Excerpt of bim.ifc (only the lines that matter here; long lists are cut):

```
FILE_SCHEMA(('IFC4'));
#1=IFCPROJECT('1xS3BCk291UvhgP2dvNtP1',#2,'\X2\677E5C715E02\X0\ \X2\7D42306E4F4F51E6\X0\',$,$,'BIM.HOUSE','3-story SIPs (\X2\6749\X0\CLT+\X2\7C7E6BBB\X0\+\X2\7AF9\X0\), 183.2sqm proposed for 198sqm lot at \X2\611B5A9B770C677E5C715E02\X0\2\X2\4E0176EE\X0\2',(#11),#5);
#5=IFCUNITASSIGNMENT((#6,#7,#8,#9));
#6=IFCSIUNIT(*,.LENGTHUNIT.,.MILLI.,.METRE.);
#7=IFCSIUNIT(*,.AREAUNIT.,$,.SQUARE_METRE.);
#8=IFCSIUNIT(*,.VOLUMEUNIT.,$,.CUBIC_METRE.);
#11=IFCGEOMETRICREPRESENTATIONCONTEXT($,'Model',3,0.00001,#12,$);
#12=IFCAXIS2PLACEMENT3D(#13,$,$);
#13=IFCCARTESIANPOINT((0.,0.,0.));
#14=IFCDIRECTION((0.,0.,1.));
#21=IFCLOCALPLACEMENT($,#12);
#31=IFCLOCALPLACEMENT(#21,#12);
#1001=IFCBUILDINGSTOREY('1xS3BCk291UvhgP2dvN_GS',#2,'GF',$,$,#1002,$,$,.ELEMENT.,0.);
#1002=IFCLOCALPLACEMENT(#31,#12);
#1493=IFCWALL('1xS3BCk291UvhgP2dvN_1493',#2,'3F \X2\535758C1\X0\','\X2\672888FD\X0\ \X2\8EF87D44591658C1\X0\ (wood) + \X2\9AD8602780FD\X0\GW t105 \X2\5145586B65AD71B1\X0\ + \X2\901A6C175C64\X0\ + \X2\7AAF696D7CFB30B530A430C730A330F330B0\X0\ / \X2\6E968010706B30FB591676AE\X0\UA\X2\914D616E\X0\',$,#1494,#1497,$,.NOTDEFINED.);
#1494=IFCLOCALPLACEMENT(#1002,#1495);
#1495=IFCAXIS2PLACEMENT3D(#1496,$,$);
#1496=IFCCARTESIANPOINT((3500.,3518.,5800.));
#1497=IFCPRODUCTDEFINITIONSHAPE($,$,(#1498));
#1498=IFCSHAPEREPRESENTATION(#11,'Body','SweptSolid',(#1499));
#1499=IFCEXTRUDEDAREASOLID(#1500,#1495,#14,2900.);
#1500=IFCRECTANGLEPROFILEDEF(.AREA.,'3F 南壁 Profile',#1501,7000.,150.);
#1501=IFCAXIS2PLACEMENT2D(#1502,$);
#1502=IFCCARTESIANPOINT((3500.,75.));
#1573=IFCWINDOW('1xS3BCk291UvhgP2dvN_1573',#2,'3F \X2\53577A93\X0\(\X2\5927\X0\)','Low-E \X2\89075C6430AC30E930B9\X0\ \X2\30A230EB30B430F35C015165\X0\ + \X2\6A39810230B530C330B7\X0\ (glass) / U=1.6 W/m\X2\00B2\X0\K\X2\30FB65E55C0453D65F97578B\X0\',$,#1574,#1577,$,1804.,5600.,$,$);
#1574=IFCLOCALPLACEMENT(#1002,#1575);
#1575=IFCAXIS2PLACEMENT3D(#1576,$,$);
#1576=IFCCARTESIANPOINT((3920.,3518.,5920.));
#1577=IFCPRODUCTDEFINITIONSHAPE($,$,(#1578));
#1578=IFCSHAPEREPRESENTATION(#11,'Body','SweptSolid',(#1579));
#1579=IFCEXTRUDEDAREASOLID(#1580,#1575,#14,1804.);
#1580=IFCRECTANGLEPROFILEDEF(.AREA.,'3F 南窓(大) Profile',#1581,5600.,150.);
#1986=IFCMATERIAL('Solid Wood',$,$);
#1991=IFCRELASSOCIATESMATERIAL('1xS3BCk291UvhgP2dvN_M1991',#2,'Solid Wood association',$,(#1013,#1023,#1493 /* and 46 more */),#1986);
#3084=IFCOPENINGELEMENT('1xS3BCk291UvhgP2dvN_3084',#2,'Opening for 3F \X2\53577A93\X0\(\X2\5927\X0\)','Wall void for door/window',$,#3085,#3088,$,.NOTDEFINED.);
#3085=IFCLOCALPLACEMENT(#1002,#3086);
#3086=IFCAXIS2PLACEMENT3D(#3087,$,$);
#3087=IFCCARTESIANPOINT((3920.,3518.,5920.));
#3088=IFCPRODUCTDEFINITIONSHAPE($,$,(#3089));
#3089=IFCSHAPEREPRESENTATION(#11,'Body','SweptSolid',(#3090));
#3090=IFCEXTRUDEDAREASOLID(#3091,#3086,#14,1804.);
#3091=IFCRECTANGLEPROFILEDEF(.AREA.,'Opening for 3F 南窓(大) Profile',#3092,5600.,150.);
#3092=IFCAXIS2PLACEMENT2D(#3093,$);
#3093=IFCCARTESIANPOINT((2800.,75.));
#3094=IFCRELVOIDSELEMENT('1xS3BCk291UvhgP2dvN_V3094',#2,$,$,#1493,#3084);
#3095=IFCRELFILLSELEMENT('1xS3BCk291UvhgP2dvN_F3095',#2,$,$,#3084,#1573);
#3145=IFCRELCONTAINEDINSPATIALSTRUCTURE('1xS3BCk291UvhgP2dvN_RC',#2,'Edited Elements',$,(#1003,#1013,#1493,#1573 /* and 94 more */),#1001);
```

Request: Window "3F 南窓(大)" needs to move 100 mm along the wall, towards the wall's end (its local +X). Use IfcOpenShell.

```python
import ifcopenshell
import ifcopenshell.api.geometry
import ifcopenshell.util.placement
import ifcopenshell.util.unit

model = ifcopenshell.open("bim.ifc")
unit_scale = ifcopenshell.util.unit.calculate_unit_scale(model)

window = model.by_guid("1xS3BCk291UvhgP2dvN_1573")
opening = window.FillsVoids[0].RelatingOpeningElement
wall = opening.VoidsElements[0].RelatingBuildingElement

wall_matrix = ifcopenshell.util.placement.get_local_placement(wall.ObjectPlacement)
shift = wall_matrix[:3, 0] * 0.1 / unit_scale
before = ifcopenshell.util.placement.get_local_placement(window.ObjectPlacement)[:3, 3].copy()

# The window is not placed relative to its opening, so move both.
for product in (opening, window):
    matrix = ifcopenshell.util.placement.get_local_placement(product.ObjectPlacement)
    matrix[:3, 3] += shift
    ifcopenshell.api.geometry.edit_object_placement(model, product=product, matrix=matrix, is_si=False)

after = ifcopenshell.util.placement.get_local_placement(window.ObjectPlacement)[:3, 3]
print("window moved by", (after - before).round(3) + 0.0)

model.write("bim_rev.ifc")
```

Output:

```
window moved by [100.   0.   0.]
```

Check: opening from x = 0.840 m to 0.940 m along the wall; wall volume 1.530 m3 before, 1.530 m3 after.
